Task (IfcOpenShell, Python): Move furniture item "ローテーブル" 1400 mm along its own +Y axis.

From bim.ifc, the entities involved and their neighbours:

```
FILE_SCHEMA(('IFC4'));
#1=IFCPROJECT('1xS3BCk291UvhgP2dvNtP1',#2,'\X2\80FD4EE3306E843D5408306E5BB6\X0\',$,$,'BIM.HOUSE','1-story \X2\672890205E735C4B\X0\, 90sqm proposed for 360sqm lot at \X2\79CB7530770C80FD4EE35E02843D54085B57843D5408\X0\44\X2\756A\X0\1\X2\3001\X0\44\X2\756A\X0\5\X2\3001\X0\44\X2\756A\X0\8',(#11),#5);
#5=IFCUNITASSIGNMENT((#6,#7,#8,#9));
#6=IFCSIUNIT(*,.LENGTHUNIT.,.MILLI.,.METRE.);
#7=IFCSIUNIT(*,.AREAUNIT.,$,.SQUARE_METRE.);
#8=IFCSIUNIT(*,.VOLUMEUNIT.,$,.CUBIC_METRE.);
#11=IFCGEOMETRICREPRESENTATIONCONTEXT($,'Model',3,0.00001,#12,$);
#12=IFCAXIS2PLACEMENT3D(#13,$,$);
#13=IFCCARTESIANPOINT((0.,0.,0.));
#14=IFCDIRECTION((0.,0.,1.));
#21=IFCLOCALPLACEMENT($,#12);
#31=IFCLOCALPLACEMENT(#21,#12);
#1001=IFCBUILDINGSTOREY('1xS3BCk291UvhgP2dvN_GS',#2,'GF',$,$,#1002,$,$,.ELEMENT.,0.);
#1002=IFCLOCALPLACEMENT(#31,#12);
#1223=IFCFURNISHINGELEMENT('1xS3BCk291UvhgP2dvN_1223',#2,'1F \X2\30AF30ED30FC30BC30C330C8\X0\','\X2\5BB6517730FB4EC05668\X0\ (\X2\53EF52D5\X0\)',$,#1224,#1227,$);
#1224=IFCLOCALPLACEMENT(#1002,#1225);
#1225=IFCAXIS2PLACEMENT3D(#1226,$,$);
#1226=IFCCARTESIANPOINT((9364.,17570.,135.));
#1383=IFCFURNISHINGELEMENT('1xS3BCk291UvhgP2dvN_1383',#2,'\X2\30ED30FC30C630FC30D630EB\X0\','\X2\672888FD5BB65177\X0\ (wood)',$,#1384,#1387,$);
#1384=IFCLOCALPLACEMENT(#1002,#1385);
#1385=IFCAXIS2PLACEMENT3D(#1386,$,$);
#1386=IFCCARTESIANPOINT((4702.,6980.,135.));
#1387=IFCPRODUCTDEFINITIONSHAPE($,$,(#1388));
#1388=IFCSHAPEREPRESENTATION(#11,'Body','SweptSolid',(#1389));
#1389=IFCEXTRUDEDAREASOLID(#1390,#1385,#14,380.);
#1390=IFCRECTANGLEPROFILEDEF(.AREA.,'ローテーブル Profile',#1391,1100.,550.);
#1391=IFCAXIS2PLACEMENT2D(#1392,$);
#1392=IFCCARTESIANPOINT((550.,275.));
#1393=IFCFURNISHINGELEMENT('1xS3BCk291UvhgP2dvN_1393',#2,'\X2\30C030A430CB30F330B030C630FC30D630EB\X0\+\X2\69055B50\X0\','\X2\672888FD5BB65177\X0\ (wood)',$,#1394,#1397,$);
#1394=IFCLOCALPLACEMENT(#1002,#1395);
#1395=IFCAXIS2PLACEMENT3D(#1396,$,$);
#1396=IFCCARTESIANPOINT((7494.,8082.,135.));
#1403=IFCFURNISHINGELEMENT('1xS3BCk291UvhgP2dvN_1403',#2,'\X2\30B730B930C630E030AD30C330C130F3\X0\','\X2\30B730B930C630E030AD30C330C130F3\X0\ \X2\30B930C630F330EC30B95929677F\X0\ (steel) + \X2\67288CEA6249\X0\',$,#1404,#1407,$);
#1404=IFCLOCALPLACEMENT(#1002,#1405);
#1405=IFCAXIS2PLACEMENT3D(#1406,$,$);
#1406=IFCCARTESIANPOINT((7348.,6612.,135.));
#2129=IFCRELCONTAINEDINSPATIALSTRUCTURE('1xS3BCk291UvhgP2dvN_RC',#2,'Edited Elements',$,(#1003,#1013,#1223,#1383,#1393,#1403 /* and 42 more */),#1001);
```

```python
import ifcopenshell
import ifcopenshell.api.geometry
import ifcopenshell.util.placement
import ifcopenshell.util.unit

model = ifcopenshell.open("bim.ifc")
unit_scale = ifcopenshell.util.unit.calculate_unit_scale(model)

item = model.by_guid("1xS3BCk291UvhgP2dvN_1383")
matrix = ifcopenshell.util.placement.get_local_placement(item.ObjectPlacement)
matrix[:3, 3] += matrix[:3, 1] * 1.4 / unit_scale
ifcopenshell.api.geometry.edit_object_placement(model, product=item, matrix=matrix, is_si=False)

print(ifcopenshell.util.placement.get_local_placement(item.ObjectPlacement).round(3) + 0.0)

model.write("bim_v2.ifc")
```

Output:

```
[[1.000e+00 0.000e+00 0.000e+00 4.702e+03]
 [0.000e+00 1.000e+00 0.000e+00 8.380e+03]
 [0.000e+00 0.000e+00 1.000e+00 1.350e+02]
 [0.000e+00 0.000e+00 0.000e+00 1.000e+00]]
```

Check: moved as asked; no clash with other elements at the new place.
